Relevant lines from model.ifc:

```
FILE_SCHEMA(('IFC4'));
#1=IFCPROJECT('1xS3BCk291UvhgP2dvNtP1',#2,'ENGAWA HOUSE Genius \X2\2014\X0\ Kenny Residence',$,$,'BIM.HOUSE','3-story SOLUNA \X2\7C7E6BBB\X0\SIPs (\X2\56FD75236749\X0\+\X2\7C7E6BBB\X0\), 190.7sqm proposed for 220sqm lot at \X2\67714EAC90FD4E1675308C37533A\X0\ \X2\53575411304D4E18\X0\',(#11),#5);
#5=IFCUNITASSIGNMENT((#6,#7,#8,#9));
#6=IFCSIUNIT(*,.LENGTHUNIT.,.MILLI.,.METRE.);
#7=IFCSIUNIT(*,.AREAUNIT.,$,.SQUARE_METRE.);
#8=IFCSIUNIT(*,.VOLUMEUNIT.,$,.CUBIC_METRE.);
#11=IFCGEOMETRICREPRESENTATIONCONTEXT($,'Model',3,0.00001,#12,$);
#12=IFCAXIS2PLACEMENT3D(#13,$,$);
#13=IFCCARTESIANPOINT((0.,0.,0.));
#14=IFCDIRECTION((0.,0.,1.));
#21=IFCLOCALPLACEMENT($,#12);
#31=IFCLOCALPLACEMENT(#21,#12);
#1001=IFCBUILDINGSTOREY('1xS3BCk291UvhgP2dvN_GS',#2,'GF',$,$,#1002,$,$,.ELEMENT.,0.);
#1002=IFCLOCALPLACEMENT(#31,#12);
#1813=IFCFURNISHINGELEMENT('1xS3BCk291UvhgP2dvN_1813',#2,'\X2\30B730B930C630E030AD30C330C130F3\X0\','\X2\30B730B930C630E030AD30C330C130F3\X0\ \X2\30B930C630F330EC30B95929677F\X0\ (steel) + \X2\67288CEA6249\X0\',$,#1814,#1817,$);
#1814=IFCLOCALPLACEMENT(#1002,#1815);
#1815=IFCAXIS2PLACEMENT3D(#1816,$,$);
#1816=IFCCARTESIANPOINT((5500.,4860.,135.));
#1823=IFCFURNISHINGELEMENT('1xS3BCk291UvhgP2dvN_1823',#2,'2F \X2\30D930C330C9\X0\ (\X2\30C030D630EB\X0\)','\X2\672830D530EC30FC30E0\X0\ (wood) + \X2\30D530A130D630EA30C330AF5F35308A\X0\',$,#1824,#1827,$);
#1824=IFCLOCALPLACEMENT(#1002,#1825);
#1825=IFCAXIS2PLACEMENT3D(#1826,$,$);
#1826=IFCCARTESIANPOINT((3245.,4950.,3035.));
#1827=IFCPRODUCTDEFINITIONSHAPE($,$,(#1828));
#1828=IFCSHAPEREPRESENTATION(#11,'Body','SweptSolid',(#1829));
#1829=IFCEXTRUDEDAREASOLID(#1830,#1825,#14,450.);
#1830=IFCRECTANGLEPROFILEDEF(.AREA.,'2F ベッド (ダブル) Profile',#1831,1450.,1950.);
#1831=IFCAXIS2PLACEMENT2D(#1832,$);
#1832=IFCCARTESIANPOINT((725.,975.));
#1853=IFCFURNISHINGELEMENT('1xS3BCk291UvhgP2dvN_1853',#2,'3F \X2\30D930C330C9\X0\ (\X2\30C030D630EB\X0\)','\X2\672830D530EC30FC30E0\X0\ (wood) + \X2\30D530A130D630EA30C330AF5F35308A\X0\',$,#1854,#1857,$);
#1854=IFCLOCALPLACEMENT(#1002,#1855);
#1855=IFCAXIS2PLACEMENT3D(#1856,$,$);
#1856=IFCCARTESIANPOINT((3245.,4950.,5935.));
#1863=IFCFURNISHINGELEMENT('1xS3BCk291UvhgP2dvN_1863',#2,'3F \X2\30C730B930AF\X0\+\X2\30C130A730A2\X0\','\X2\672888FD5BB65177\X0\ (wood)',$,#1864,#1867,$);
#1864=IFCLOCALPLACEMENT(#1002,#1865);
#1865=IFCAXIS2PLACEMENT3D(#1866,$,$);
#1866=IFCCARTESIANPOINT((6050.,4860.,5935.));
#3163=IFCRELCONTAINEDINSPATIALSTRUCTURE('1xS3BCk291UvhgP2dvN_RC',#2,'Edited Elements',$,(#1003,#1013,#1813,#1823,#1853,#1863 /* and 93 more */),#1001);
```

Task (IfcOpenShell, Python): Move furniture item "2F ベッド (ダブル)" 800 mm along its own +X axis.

```python
import ifcopenshell
import ifcopenshell.api.geometry
import ifcopenshell.util.placement

model = ifcopenshell.open("model.ifc")

item = model.by_guid("1xS3BCk291UvhgP2dvN_1823")
matrix = ifcopenshell.util.placement.get_local_placement(item.ObjectPlacement)
matrix[:3, 3] += matrix[:3, 0] * 800.0
ifcopenshell.api.geometry.edit_object_placement(model, product=item, matrix=matrix, is_si=False)

print(ifcopenshell.util.placement.get_local_placement(item.ObjectPlacement).round(3) + 0.0)

model.write("model_edited.ifc")
```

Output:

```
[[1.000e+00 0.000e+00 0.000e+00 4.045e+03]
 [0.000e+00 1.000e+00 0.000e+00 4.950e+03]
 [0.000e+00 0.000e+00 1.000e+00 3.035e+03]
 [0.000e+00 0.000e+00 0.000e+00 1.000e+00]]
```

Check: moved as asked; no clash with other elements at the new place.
